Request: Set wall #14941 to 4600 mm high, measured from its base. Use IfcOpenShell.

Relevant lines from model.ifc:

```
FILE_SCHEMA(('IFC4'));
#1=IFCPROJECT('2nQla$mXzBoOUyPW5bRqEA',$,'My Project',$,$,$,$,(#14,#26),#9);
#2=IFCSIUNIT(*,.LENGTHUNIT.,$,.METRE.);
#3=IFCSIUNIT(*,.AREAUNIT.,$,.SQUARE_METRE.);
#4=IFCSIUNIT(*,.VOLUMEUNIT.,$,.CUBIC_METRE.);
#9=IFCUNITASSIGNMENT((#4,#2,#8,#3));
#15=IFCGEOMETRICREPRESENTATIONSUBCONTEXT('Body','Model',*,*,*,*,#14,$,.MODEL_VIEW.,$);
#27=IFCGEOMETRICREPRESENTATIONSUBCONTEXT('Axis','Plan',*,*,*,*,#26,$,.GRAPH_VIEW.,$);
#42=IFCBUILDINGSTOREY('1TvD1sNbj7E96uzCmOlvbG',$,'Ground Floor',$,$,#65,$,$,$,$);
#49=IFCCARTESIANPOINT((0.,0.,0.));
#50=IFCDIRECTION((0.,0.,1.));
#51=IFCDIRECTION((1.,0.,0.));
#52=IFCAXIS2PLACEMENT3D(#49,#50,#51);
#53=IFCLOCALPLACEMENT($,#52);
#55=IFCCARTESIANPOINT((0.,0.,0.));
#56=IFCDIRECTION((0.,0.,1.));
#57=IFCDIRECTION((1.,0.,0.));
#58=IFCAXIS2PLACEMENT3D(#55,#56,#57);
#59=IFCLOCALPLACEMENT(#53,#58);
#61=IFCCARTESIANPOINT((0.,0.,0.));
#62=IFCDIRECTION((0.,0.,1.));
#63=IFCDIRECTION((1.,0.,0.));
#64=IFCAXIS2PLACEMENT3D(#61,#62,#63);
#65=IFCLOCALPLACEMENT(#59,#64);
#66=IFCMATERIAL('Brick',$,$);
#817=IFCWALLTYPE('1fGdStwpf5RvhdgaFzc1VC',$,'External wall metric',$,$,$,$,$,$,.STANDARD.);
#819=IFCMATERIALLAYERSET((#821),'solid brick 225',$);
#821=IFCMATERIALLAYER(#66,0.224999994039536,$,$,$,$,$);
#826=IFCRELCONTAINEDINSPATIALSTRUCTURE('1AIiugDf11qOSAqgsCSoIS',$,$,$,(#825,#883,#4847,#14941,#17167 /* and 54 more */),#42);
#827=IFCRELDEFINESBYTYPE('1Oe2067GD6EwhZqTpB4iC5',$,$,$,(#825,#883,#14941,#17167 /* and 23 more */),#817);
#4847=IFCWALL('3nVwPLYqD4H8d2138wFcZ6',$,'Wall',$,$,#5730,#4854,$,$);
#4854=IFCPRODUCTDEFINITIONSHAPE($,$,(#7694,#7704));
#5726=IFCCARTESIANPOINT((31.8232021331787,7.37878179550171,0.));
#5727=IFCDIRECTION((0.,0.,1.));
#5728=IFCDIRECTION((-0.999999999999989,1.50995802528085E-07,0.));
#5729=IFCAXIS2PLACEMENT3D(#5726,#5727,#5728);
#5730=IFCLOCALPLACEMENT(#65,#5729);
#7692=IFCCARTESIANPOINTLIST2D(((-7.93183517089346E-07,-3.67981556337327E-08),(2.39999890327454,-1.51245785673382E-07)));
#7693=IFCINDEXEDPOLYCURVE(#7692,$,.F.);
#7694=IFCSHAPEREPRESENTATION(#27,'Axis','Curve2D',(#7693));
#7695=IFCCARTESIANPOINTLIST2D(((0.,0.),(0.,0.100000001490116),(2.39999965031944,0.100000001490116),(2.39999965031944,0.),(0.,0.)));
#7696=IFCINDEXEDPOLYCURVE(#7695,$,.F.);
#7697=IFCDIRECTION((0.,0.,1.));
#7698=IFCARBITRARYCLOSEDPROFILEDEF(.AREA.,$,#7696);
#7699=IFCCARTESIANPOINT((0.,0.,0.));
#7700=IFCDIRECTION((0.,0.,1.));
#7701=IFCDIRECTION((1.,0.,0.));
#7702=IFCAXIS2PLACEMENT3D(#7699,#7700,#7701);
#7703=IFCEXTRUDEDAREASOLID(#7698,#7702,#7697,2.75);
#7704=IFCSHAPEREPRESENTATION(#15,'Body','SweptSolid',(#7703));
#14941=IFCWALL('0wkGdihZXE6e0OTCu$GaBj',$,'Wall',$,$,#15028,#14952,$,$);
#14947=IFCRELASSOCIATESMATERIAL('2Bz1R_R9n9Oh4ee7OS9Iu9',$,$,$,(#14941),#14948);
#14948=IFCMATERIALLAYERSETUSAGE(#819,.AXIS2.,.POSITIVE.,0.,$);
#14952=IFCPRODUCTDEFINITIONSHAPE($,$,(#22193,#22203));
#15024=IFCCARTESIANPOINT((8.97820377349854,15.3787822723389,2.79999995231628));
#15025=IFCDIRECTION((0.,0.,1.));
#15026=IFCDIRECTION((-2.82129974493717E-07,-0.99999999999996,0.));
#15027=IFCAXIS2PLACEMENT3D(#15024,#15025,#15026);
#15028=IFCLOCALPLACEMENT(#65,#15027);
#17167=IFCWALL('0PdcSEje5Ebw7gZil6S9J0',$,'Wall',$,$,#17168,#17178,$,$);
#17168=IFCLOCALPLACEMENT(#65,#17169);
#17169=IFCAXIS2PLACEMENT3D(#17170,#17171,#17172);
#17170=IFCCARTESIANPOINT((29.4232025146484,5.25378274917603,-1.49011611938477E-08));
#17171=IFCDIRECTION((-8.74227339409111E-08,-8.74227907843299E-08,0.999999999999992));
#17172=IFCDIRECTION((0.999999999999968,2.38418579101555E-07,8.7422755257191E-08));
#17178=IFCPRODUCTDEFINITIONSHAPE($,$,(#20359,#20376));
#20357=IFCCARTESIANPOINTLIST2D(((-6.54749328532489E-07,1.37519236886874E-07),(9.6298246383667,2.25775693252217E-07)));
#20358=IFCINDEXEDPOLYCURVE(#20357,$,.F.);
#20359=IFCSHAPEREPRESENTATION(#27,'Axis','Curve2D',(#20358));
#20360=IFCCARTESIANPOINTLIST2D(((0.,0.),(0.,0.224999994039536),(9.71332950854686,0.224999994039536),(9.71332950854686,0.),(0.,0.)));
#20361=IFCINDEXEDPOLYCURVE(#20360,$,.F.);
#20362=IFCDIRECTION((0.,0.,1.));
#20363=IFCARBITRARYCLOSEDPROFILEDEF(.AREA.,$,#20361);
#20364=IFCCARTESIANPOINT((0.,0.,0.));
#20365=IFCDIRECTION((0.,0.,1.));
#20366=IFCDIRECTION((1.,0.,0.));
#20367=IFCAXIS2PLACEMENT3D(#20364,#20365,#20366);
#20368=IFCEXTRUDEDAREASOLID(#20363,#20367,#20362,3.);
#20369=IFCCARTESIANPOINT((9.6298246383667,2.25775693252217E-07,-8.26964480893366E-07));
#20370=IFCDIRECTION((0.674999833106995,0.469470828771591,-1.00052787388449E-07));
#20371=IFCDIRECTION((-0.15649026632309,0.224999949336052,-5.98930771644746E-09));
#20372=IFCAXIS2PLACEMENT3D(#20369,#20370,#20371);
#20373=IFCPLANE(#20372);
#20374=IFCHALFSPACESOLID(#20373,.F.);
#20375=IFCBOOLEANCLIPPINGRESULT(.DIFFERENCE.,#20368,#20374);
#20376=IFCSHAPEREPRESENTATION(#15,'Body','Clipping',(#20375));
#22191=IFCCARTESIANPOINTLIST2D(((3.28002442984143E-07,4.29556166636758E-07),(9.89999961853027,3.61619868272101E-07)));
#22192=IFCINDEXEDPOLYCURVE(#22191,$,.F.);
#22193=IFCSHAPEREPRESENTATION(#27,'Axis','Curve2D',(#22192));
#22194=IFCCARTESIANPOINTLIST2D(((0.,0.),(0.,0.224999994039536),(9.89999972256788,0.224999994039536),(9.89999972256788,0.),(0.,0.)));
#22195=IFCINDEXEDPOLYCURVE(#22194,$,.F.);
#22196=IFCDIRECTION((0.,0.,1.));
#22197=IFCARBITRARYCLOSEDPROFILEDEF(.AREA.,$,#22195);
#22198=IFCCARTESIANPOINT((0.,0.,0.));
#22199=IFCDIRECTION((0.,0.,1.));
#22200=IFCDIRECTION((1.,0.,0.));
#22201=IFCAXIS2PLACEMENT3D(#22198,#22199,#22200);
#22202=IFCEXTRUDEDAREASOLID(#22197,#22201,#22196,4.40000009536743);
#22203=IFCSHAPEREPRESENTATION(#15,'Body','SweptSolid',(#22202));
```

```python
import ifcopenshell
import ifcopenshell.geom
import ifcopenshell.util.representation
import ifcopenshell.util.shape
import ifcopenshell.util.unit

model = ifcopenshell.open("model.ifc")
unit_scale = ifcopenshell.util.unit.calculate_unit_scale(model)
settings = ifcopenshell.geom.settings()


def volume(element):
    """Net volume in cubic metres, openings subtracted."""
    shape = ifcopenshell.geom.create_shape(settings, element)
    return ifcopenshell.util.shape.get_volume(shape.geometry)


wall = model.by_guid("0wkGdihZXE6e0OTCu$GaBj")
before = volume(wall)

body = ifcopenshell.util.representation.get_representation(wall, "Model", "Body")
solid = body.Items[0]
old_height = solid.Depth
solid.Depth = 4.6 / unit_scale
after = volume(wall)

print(f"height {old_height:g} -> {solid.Depth:g}, volume {before:.3f} -> {after:.3f} m3")

model.write("model_rev.ifc")
```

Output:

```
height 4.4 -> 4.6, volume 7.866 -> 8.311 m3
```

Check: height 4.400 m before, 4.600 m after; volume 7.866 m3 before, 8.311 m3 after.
